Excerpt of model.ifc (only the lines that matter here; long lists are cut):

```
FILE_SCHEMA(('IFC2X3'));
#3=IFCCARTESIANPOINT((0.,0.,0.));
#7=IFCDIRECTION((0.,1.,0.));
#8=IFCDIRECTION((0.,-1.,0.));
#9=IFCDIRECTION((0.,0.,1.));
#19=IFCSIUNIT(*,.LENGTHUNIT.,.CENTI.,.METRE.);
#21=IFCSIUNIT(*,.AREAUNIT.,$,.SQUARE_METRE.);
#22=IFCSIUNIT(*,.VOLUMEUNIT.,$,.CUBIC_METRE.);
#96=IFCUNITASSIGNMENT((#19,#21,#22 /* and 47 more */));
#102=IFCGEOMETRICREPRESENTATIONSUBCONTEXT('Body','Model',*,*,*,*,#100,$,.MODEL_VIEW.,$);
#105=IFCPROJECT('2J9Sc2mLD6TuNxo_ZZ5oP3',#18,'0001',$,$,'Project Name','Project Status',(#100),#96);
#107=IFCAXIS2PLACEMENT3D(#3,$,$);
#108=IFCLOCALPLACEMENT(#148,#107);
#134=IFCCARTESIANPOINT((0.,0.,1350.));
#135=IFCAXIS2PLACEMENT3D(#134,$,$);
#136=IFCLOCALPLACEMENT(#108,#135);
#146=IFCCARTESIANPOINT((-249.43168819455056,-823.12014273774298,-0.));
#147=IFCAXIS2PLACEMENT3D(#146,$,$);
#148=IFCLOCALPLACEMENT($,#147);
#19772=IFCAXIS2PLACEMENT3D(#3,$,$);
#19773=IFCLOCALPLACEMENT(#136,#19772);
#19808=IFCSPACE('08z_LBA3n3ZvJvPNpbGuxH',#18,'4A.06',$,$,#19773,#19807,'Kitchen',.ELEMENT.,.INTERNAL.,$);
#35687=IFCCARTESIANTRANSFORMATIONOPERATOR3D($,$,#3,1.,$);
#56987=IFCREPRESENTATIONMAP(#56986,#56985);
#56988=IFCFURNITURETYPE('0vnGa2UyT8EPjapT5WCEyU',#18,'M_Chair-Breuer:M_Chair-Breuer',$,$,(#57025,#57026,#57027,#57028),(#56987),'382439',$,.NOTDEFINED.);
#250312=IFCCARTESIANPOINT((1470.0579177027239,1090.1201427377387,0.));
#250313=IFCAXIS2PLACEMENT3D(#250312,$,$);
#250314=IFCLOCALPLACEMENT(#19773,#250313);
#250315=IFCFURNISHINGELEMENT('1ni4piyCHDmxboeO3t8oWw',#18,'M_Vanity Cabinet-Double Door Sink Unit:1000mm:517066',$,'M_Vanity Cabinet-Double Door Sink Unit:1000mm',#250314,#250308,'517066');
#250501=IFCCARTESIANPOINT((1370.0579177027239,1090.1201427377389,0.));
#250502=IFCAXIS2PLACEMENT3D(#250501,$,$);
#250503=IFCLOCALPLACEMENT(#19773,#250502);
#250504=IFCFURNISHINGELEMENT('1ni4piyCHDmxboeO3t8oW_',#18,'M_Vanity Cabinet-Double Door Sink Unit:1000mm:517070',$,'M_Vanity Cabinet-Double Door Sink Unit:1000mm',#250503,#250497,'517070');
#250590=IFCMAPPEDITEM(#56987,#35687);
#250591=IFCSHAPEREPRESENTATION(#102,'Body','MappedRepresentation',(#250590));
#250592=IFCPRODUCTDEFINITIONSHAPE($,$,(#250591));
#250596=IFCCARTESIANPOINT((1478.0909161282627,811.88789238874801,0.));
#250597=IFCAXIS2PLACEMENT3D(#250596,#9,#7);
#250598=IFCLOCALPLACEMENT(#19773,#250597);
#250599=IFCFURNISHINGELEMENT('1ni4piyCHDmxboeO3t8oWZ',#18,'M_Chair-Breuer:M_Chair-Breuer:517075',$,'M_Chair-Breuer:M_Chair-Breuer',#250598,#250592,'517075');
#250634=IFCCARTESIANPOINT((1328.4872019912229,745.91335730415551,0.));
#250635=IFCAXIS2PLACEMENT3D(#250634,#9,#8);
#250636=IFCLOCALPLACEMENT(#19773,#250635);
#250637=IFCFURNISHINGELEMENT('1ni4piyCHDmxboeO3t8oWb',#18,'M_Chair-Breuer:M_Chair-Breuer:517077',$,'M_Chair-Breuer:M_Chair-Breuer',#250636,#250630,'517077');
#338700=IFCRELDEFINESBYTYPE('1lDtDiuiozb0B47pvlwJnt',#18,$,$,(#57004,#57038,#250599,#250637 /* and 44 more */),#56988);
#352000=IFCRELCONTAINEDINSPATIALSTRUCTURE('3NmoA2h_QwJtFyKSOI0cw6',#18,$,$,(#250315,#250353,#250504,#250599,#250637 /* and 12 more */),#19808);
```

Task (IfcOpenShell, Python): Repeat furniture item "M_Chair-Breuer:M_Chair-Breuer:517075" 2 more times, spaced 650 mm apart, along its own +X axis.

```python
import ifcopenshell
import ifcopenshell.api.geometry
import ifcopenshell.api.root
import ifcopenshell.util.element
import ifcopenshell.util.placement
import ifcopenshell.util.unit

model = ifcopenshell.open("model.ifc")
unit_scale = ifcopenshell.util.unit.calculate_unit_scale(model)


def reuse_history(source, copy):
    """copy_class also copies each property set's owner history, people and application; keep the originals."""
    for rel in copy.IsDefinedBy:
        if rel.is_a("IfcRelDefinesByProperties") and (history := rel.RelatingPropertyDefinition.OwnerHistory):
            rel.RelatingPropertyDefinition.OwnerHistory = source.OwnerHistory
            ifcopenshell.util.element.remove_deep2(model, history)


source = model.by_id(250599)
base = ifcopenshell.util.placement.get_local_placement(source.ObjectPlacement)
step = base[:3, 0] * 0.65 / unit_scale

for i in range(1, 3):
    copy = ifcopenshell.api.root.copy_class(model, product=source)
    copy.Representation = ifcopenshell.util.element.copy_deep(
        model, source.Representation, exclude=["IfcGeometricRepresentationContext", "IfcRepresentationMap"]
    )
    copy.Name = "M_Chair-Breuer:M_Chair-Breuer"
    copy.Tag = None
    reuse_history(source, copy)
    matrix = base.copy()
    matrix[:3, 3] += i * step
    print("added at", matrix[:3, 3].round(3) + 0.0)
    ifcopenshell.api.geometry.edit_object_placement(model, product=copy, matrix=matrix, is_si=False)

model.write("model_v2.ifc")
```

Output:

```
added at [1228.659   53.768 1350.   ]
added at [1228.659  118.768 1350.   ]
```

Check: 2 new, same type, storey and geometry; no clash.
